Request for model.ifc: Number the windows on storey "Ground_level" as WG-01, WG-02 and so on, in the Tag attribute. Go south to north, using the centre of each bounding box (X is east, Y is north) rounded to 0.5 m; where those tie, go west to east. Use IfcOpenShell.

First a look at what the model holds.

```python
import ifcopenshell
import ifcopenshell.util.element
import ifcopenshell.util.placement

model = ifcopenshell.open("model.ifc")
print(model.schema)
storey = next(s for s in model.by_type("IfcBuildingStorey") if s.Name == "Ground_level")
windows = [e for e in ifcopenshell.util.element.get_decomposition(storey) if e.is_a("IfcWindow")]
for e in sorted(windows, key=lambda e: e.id()):
    origin = ifcopenshell.util.placement.get_local_placement(e.ObjectPlacement)[:3, 3]
    print(e.id(), e.Tag, e.Name, origin.round(2) + 0.0, sep=" | ")
```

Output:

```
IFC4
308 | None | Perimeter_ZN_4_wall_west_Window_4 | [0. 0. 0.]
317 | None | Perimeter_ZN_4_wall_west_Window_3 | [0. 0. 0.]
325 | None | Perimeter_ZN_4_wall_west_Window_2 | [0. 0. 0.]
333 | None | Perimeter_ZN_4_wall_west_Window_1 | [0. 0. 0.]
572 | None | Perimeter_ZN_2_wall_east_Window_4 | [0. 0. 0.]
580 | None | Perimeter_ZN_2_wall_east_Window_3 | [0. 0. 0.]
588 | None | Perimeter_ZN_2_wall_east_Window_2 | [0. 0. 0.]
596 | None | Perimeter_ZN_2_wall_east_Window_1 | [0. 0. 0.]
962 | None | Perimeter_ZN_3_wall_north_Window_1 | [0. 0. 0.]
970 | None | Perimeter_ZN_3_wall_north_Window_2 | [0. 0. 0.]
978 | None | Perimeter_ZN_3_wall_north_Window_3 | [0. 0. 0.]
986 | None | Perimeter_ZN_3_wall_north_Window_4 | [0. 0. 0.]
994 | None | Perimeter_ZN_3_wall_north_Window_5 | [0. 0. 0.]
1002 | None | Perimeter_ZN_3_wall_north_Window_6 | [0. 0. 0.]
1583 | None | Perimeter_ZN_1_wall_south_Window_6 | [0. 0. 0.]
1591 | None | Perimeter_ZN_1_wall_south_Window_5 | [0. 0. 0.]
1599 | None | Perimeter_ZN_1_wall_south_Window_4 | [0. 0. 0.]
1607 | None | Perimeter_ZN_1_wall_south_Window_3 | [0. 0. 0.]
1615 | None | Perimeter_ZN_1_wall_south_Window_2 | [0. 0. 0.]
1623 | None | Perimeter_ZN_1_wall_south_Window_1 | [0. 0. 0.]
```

```python
import ifcopenshell
import ifcopenshell.geom
import ifcopenshell.util.element
import ifcopenshell.util.shape

model = ifcopenshell.open("model.ifc")
settings = ifcopenshell.geom.settings()
settings.set("use-world-coords", True)


def centre(element):
    shape = ifcopenshell.geom.create_shape(settings, element)
    return ifcopenshell.util.shape.get_bbox_centroid(shape.geometry)


storey = next(s for s in model.by_type("IfcBuildingStorey") if s.Name == "Ground_level")
windows = [e for e in ifcopenshell.util.element.get_decomposition(storey) if e.is_a("IfcWindow")]

# Insertion points can sit at a corner or the storey origin, so sort by the geometry (in metres).
centres = {e: centre(e) for e in windows}
windows.sort(key=lambda e: (round(centres[e][1] / 0.5), centres[e][0]))

for i, e in enumerate(windows, start=1):
    number = f"WG-{i:02d}"
    e.Tag = number
    print(e.id(), number)

model.write("model_edited.ifc")
```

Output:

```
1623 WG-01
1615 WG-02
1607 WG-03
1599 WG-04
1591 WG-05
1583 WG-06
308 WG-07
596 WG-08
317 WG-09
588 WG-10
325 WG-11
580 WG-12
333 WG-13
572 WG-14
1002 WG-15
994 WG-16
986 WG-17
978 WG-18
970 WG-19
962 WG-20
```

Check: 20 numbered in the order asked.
